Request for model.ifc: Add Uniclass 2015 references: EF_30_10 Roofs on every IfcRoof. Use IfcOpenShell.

First a look at what the model holds.

```python
import ifcopenshell

model = ifcopenshell.open("model.ifc")
print(model.schema)
print("classifications:", [c.Name for c in model.by_type("IfcClassification")])
for ifc_class in ("IfcDoor", "IfcRoof", "IfcStair", "IfcWall", "IfcWindow"):
    print(ifc_class, len(model.by_type(ifc_class)))
```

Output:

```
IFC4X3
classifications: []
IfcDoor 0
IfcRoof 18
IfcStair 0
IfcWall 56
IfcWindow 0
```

```python
import ifcopenshell
import ifcopenshell.api.classification

model = ifcopenshell.open("model.ifc")

system = ifcopenshell.api.classification.add_classification(model, classification="Uniclass 2015")

codes = {
    "IfcRoof": ("EF_30_10", "Roofs"),
}
for ifc_class, (code, name) in codes.items():
    products = model.by_type(ifc_class)
    ifcopenshell.api.classification.add_reference(
        model, products=products, classification=system, identification=code, name=name
    )
    print(code, len(products))

model.write("model_edited.ifc")
```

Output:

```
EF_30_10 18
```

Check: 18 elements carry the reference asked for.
